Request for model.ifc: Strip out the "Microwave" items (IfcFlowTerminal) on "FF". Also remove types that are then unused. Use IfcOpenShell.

First a look at what the model holds.

```python
import ifcopenshell
import ifcopenshell.util.element

model = ifcopenshell.open("model.ifc")
print(model.schema)
storey = next(s for s in model.by_type("IfcBuildingStorey") if s.Name == "FF")
terminals = [e for e in ifcopenshell.util.element.get_decomposition(storey) if e.is_a("IfcFlowTerminal")]
seen = {}
for e in terminals:
    element_type = ifcopenshell.util.element.get_type(e)
    name = element_type.Name if element_type not in (None, e) else None
    seen[name] = seen.get(name, 0) + 1
for name, count in sorted(seen.items(), key=str):
    print(count, "x", name)
```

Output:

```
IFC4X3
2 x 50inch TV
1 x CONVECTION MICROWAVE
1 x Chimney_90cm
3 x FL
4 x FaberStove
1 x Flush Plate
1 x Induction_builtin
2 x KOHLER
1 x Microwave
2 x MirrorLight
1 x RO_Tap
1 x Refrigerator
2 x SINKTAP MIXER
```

```python
import ifcopenshell
import ifcopenshell.api.root
import ifcopenshell.util.element

model = ifcopenshell.open("model.ifc")

storey = next(s for s in model.by_type("IfcBuildingStorey") if s.Name == "FF")
terminals = [e for e in ifcopenshell.util.element.get_decomposition(storey) if e.is_a("IfcFlowTerminal")]
targets = [e for e in terminals if (t := ifcopenshell.util.element.get_type(e)) not in (None, e) and t.Name == "Microwave"]
types = {ifcopenshell.util.element.get_type(e) for e in targets} - {None, *targets}

for e in targets:
    ifcopenshell.api.root.remove_product(model, product=e)
print(len(targets), "removed")

unused = [t for t in types if not ifcopenshell.util.element.get_types(t)]
for t in unused:
    ifcopenshell.api.root.remove_product(model, product=t)
print(len(unused), "unused types removed")

model.write("model_rev.ifc")
```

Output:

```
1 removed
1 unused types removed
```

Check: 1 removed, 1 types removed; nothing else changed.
